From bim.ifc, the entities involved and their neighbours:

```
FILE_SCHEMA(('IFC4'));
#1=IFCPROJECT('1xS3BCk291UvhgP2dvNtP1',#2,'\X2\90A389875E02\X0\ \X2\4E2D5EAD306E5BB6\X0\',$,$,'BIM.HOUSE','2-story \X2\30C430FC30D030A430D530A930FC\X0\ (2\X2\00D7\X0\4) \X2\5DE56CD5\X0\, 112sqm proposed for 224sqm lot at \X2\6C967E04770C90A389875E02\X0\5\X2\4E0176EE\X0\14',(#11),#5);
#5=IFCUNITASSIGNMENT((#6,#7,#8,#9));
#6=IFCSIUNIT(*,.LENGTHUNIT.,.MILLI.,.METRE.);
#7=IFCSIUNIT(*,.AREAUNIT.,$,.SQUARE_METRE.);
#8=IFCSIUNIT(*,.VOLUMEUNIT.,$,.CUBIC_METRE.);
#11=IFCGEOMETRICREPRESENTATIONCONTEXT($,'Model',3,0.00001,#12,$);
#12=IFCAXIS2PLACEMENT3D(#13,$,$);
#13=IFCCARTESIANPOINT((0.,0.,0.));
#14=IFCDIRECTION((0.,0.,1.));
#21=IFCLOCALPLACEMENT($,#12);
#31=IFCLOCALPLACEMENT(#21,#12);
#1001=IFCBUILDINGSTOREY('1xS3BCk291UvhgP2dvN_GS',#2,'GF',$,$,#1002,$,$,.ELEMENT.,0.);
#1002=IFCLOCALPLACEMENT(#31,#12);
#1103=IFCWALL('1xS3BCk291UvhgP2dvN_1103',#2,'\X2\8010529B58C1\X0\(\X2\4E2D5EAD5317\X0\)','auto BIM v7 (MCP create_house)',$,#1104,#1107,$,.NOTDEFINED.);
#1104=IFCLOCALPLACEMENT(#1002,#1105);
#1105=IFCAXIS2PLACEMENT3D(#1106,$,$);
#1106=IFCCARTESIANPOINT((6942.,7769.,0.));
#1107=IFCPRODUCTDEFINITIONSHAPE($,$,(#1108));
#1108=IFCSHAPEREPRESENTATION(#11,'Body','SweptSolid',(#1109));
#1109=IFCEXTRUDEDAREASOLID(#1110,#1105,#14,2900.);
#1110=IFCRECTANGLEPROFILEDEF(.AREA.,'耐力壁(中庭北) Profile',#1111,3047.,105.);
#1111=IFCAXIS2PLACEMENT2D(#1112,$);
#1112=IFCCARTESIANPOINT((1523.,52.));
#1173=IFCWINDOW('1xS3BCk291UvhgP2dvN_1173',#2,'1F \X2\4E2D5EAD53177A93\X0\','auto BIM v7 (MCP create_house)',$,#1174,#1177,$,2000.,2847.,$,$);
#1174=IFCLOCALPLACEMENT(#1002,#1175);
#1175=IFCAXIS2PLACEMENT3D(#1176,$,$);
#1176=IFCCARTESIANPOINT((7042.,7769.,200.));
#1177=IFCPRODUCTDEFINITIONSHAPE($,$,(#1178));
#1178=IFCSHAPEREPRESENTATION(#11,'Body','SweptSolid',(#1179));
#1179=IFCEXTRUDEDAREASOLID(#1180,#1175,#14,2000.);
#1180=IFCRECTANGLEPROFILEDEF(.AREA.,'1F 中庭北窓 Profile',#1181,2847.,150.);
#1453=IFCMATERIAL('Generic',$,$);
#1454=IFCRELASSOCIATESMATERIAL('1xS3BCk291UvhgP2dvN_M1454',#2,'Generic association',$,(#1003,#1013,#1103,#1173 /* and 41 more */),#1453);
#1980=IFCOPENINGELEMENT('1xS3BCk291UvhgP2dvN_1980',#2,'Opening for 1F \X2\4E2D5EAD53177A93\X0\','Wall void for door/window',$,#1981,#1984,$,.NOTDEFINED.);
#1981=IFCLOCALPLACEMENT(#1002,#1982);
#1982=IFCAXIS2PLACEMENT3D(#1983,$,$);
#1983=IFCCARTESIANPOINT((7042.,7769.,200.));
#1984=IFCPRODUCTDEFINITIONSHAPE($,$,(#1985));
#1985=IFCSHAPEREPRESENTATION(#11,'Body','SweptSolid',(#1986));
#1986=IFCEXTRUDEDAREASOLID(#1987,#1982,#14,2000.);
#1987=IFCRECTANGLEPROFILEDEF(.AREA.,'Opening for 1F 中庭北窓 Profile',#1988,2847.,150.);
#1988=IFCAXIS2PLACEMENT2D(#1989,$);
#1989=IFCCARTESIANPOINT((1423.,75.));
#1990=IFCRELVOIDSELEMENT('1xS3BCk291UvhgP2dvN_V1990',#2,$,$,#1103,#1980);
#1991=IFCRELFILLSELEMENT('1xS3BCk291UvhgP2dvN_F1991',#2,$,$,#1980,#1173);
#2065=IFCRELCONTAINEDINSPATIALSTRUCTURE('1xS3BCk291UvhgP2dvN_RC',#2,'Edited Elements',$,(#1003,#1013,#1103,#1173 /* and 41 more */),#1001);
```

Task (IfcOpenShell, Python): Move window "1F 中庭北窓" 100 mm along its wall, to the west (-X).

```python
import ifcopenshell
import ifcopenshell.api.geometry
import ifcopenshell.util.placement
import ifcopenshell.util.unit

model = ifcopenshell.open("bim.ifc")
unit_scale = ifcopenshell.util.unit.calculate_unit_scale(model)

window = model.by_guid("1xS3BCk291UvhgP2dvN_1173")
opening = window.FillsVoids[0].RelatingOpeningElement
wall = opening.VoidsElements[0].RelatingBuildingElement

wall_matrix = ifcopenshell.util.placement.get_local_placement(wall.ObjectPlacement)
shift = wall_matrix[:3, 0] * -0.1 / unit_scale
before = ifcopenshell.util.placement.get_local_placement(window.ObjectPlacement)[:3, 3].copy()

# The window is not placed relative to its opening, so move both.
for product in (opening, window):
    matrix = ifcopenshell.util.placement.get_local_placement(product.ObjectPlacement)
    matrix[:3, 3] += shift
    ifcopenshell.api.geometry.edit_object_placement(model, product=product, matrix=matrix, is_si=False)

after = ifcopenshell.util.placement.get_local_placement(window.ObjectPlacement)[:3, 3]
print("window moved by", (after - before).round(3) + 0.0)

model.write("bim_rev.ifc")
```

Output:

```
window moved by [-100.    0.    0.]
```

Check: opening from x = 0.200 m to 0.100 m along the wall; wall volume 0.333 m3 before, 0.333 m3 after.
